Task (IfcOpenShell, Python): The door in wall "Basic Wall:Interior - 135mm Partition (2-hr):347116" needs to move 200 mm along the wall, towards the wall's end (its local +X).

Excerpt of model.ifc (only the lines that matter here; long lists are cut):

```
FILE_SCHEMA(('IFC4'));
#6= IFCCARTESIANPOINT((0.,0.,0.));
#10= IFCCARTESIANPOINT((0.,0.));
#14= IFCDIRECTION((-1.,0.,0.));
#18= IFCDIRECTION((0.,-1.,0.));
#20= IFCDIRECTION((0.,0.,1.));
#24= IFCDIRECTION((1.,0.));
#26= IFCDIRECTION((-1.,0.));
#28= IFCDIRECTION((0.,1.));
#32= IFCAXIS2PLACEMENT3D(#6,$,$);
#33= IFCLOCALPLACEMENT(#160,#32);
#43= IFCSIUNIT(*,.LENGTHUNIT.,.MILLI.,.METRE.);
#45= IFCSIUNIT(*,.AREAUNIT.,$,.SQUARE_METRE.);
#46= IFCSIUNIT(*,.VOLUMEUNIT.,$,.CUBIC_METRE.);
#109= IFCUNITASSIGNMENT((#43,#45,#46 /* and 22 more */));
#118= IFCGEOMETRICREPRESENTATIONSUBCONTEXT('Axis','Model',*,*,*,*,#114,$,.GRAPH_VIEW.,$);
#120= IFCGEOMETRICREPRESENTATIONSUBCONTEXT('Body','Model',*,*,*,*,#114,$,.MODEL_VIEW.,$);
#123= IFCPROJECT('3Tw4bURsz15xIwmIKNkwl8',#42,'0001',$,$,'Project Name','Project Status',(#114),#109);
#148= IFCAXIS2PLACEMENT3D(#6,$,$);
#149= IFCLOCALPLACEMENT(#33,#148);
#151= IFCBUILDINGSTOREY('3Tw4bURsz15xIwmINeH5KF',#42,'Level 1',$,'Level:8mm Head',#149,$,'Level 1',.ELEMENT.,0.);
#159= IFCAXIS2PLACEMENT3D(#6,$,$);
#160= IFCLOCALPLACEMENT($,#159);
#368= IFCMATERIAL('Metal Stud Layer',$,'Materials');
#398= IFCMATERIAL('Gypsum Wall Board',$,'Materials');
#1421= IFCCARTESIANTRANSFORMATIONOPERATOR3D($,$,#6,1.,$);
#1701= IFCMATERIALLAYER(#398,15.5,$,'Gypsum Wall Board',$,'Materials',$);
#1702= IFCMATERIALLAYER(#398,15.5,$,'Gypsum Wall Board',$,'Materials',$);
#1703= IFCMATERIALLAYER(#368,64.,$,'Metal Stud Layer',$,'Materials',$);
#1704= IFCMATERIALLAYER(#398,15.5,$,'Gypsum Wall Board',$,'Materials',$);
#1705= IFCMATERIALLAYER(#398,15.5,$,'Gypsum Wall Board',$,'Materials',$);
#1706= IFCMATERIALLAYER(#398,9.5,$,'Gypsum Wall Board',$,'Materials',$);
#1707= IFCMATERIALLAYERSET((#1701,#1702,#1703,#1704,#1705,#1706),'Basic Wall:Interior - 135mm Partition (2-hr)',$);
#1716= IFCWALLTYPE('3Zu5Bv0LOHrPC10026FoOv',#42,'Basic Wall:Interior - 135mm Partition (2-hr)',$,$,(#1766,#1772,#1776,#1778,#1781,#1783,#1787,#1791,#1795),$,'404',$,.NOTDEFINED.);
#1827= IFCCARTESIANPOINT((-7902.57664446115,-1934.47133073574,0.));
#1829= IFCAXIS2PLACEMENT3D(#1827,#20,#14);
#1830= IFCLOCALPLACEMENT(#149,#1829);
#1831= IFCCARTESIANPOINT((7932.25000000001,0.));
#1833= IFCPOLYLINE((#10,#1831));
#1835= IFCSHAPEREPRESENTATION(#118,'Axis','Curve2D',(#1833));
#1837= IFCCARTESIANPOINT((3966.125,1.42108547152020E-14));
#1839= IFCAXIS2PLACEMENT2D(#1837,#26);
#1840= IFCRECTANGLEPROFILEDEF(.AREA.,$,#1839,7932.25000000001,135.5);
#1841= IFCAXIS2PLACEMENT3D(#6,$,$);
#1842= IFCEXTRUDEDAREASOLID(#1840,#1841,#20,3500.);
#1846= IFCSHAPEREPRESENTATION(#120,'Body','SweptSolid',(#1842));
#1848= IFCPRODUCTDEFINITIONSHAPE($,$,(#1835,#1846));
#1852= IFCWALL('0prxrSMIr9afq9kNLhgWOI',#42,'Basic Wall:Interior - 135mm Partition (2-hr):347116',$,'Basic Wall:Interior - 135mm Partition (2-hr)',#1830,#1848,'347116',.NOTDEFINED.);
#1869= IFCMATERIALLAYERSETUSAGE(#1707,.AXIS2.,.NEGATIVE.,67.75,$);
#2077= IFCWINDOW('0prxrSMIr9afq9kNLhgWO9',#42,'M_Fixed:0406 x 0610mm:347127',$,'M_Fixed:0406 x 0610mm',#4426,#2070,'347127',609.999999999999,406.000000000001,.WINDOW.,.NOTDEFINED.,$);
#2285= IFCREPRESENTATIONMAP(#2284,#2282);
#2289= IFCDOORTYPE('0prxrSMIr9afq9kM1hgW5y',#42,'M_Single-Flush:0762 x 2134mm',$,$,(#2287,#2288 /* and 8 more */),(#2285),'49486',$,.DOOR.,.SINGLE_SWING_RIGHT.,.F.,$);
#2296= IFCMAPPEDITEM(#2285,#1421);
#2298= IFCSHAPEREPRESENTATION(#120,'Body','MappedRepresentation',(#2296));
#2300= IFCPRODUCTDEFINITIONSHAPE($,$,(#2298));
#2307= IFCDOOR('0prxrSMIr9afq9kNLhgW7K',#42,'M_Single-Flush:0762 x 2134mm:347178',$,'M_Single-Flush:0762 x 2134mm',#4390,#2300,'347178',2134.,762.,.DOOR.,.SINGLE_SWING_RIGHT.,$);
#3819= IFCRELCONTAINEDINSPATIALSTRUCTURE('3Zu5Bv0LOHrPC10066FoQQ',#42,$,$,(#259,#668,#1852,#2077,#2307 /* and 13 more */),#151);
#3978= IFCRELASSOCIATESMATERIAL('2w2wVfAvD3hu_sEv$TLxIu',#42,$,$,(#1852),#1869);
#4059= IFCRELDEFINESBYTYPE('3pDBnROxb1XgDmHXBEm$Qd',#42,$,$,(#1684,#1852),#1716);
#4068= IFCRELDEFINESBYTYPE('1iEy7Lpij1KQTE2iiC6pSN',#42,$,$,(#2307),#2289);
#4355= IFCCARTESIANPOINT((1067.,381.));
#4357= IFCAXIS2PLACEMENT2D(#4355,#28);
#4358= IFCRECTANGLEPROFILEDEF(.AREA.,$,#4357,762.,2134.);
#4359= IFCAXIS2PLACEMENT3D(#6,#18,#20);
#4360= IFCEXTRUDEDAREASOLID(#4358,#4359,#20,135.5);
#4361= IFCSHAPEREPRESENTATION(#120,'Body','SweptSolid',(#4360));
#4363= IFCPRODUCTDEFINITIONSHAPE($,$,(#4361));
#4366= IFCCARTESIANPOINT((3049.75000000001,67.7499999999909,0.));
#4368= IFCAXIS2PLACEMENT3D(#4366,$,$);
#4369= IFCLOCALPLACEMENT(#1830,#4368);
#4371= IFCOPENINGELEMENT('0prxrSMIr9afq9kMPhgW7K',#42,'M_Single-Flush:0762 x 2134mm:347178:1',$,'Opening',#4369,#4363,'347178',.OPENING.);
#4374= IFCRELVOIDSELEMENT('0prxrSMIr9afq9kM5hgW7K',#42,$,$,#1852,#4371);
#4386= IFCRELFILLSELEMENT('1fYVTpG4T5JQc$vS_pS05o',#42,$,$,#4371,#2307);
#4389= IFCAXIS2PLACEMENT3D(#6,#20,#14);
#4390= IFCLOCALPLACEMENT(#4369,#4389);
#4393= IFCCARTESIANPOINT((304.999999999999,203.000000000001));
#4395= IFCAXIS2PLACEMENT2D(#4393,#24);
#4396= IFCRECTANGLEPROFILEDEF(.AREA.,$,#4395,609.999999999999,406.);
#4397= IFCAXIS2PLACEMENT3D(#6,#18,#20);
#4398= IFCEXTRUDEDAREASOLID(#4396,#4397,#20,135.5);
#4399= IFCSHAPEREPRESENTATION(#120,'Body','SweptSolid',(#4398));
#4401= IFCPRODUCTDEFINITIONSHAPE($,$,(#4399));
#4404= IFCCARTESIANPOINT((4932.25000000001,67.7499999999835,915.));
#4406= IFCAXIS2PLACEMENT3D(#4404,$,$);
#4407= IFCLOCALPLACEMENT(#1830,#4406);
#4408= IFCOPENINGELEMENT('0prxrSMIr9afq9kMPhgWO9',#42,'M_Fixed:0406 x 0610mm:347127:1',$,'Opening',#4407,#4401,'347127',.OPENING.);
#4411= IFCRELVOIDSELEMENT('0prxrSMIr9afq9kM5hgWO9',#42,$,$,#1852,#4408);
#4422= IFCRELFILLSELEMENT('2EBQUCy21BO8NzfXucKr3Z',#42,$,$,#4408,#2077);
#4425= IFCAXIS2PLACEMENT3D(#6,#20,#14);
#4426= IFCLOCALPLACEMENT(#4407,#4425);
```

```python
import ifcopenshell
import ifcopenshell.api.geometry
import ifcopenshell.util.placement

model = ifcopenshell.open("model.ifc")

door = model.by_guid("0prxrSMIr9afq9kNLhgW7K")
opening = door.FillsVoids[0].RelatingOpeningElement
wall = opening.VoidsElements[0].RelatingBuildingElement

wall_matrix = ifcopenshell.util.placement.get_local_placement(wall.ObjectPlacement)
shift = wall_matrix[:3, 0] * 200.0
before = ifcopenshell.util.placement.get_local_placement(door.ObjectPlacement)[:3, 3].copy()

# The door is placed relative to its opening, so it follows when the opening moves.
matrix = ifcopenshell.util.placement.get_local_placement(opening.ObjectPlacement)
matrix[:3, 3] += shift
ifcopenshell.api.geometry.edit_object_placement(
    model, product=opening, matrix=matrix, is_si=False, should_transform_children=True
)

after = ifcopenshell.util.placement.get_local_placement(door.ObjectPlacement)[:3, 3]
print("door moved by", (after - before).round(3) + 0.0)

model.write("model-out.ifc")
```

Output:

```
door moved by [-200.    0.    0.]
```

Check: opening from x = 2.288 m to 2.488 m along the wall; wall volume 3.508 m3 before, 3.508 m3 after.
